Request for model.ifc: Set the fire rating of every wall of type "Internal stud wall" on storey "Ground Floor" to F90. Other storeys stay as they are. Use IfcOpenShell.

First a look at what the model holds.

```python
import ifcopenshell
import ifcopenshell.util.element

model = ifcopenshell.open("model.ifc")
print(model.schema)
storey = next(s for s in model.by_type("IfcBuildingStorey") if s.Name == "Ground Floor")
walls = [e for e in ifcopenshell.util.element.get_decomposition(storey) if e.is_a("IfcWall")]
seen = {}
for e in walls:
    element_type = ifcopenshell.util.element.get_type(e)
    key = (element_type.Name if element_type != e and element_type else None, ifcopenshell.util.element.get_pset(e, "Pset_WallCommon", "FireRating"))
    seen[key] = seen.get(key, 0) + 1
for (name, value), count in sorted(seen.items(), key=str):
    print(count, "x", name, "|", value)
```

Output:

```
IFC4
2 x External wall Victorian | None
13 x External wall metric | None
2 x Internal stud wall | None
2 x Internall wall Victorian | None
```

```python
import ifcopenshell
import ifcopenshell.api.pset
import ifcopenshell.util.element

model = ifcopenshell.open("model.ifc")

storey = next(s for s in model.by_type("IfcBuildingStorey") if s.Name == "Ground Floor")
walls = [e for e in ifcopenshell.util.element.get_decomposition(storey) if e.is_a("IfcWall")]

count = 0
for e in walls:
    element_type = ifcopenshell.util.element.get_type(e)
    if element_type in (None, e) or element_type.Name != "Internal stud wall":
        continue
    # add_pset returns the element's existing set when there is one.
    pset = ifcopenshell.api.pset.add_pset(model, product=e, name="Pset_WallCommon")
    ifcopenshell.api.pset.edit_pset(model, pset=pset, properties={"FireRating": "F90"})
    count += 1

print(count, "walls updated")

model.write("model_rev.ifc")
```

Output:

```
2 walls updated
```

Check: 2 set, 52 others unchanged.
